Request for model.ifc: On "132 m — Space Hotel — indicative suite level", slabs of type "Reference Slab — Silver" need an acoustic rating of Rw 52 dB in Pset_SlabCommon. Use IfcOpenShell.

First a look at what the model holds.

```python
import ifcopenshell
import ifcopenshell.util.element

model = ifcopenshell.open("model.ifc")
print(model.schema)
storey = next(s for s in model.by_type("IfcBuildingStorey") if s.Name == "132 m — Space Hotel — indicative suite level")
slabs = [e for e in ifcopenshell.util.element.get_decomposition(storey) if e.is_a("IfcSlab")]
seen = {}
for e in slabs:
    element_type = ifcopenshell.util.element.get_type(e)
    key = (element_type.Name if element_type != e and element_type else None, ifcopenshell.util.element.get_pset(e, "Pset_SlabCommon", "AcousticRating"))
    seen[key] = seen.get(key, 0) + 1
for (name, value), count in sorted(seen.items(), key=str):
    print(count, "x", name, "|", value)
```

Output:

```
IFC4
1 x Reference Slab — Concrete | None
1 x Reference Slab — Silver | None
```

```python
import ifcopenshell
import ifcopenshell.api.pset
import ifcopenshell.util.element

model = ifcopenshell.open("model.ifc")

storey = next(s for s in model.by_type("IfcBuildingStorey") if s.Name == "132 m — Space Hotel — indicative suite level")
slabs = [e for e in ifcopenshell.util.element.get_decomposition(storey) if e.is_a("IfcSlab")]

count = 0
for e in slabs:
    element_type = ifcopenshell.util.element.get_type(e)
    if element_type in (None, e) or element_type.Name != "Reference Slab — Silver":
        continue
    # add_pset returns the element's existing set when there is one.
    pset = ifcopenshell.api.pset.add_pset(model, product=e, name="Pset_SlabCommon")
    ifcopenshell.api.pset.edit_pset(model, pset=pset, properties={"AcousticRating": "Rw 52 dB"})
    count += 1

print(count, "slabs updated")

model.write("model_edited.ifc")
```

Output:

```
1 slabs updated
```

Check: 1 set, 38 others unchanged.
